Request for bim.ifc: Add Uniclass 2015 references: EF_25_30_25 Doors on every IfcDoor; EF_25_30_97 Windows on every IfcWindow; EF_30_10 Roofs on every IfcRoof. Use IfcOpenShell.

First a look at what the model holds.

```python
import ifcopenshell

model = ifcopenshell.open("bim.ifc")
print(model.schema)
print("classifications:", [c.Name for c in model.by_type("IfcClassification")])
for ifc_class in ("IfcDoor", "IfcRoof", "IfcStair", "IfcWall", "IfcWindow"):
    print(ifc_class, len(model.by_type(ifc_class)))
```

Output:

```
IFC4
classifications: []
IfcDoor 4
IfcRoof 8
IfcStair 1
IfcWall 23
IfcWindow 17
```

```python
import ifcopenshell
import ifcopenshell.api.classification

model = ifcopenshell.open("bim.ifc")

system = ifcopenshell.api.classification.add_classification(model, classification="Uniclass 2015")

codes = {
    "IfcDoor": ("EF_25_30_25", "Doors"),
    "IfcWindow": ("EF_25_30_97", "Windows"),
    "IfcRoof": ("EF_30_10", "Roofs"),
}
for ifc_class, (code, name) in codes.items():
    products = model.by_type(ifc_class)
    ifcopenshell.api.classification.add_reference(
        model, products=products, classification=system, identification=code, name=name
    )
    print(code, len(products))

model.write("bim_edited.ifc")
```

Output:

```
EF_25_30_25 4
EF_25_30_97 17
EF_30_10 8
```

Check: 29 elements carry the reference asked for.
